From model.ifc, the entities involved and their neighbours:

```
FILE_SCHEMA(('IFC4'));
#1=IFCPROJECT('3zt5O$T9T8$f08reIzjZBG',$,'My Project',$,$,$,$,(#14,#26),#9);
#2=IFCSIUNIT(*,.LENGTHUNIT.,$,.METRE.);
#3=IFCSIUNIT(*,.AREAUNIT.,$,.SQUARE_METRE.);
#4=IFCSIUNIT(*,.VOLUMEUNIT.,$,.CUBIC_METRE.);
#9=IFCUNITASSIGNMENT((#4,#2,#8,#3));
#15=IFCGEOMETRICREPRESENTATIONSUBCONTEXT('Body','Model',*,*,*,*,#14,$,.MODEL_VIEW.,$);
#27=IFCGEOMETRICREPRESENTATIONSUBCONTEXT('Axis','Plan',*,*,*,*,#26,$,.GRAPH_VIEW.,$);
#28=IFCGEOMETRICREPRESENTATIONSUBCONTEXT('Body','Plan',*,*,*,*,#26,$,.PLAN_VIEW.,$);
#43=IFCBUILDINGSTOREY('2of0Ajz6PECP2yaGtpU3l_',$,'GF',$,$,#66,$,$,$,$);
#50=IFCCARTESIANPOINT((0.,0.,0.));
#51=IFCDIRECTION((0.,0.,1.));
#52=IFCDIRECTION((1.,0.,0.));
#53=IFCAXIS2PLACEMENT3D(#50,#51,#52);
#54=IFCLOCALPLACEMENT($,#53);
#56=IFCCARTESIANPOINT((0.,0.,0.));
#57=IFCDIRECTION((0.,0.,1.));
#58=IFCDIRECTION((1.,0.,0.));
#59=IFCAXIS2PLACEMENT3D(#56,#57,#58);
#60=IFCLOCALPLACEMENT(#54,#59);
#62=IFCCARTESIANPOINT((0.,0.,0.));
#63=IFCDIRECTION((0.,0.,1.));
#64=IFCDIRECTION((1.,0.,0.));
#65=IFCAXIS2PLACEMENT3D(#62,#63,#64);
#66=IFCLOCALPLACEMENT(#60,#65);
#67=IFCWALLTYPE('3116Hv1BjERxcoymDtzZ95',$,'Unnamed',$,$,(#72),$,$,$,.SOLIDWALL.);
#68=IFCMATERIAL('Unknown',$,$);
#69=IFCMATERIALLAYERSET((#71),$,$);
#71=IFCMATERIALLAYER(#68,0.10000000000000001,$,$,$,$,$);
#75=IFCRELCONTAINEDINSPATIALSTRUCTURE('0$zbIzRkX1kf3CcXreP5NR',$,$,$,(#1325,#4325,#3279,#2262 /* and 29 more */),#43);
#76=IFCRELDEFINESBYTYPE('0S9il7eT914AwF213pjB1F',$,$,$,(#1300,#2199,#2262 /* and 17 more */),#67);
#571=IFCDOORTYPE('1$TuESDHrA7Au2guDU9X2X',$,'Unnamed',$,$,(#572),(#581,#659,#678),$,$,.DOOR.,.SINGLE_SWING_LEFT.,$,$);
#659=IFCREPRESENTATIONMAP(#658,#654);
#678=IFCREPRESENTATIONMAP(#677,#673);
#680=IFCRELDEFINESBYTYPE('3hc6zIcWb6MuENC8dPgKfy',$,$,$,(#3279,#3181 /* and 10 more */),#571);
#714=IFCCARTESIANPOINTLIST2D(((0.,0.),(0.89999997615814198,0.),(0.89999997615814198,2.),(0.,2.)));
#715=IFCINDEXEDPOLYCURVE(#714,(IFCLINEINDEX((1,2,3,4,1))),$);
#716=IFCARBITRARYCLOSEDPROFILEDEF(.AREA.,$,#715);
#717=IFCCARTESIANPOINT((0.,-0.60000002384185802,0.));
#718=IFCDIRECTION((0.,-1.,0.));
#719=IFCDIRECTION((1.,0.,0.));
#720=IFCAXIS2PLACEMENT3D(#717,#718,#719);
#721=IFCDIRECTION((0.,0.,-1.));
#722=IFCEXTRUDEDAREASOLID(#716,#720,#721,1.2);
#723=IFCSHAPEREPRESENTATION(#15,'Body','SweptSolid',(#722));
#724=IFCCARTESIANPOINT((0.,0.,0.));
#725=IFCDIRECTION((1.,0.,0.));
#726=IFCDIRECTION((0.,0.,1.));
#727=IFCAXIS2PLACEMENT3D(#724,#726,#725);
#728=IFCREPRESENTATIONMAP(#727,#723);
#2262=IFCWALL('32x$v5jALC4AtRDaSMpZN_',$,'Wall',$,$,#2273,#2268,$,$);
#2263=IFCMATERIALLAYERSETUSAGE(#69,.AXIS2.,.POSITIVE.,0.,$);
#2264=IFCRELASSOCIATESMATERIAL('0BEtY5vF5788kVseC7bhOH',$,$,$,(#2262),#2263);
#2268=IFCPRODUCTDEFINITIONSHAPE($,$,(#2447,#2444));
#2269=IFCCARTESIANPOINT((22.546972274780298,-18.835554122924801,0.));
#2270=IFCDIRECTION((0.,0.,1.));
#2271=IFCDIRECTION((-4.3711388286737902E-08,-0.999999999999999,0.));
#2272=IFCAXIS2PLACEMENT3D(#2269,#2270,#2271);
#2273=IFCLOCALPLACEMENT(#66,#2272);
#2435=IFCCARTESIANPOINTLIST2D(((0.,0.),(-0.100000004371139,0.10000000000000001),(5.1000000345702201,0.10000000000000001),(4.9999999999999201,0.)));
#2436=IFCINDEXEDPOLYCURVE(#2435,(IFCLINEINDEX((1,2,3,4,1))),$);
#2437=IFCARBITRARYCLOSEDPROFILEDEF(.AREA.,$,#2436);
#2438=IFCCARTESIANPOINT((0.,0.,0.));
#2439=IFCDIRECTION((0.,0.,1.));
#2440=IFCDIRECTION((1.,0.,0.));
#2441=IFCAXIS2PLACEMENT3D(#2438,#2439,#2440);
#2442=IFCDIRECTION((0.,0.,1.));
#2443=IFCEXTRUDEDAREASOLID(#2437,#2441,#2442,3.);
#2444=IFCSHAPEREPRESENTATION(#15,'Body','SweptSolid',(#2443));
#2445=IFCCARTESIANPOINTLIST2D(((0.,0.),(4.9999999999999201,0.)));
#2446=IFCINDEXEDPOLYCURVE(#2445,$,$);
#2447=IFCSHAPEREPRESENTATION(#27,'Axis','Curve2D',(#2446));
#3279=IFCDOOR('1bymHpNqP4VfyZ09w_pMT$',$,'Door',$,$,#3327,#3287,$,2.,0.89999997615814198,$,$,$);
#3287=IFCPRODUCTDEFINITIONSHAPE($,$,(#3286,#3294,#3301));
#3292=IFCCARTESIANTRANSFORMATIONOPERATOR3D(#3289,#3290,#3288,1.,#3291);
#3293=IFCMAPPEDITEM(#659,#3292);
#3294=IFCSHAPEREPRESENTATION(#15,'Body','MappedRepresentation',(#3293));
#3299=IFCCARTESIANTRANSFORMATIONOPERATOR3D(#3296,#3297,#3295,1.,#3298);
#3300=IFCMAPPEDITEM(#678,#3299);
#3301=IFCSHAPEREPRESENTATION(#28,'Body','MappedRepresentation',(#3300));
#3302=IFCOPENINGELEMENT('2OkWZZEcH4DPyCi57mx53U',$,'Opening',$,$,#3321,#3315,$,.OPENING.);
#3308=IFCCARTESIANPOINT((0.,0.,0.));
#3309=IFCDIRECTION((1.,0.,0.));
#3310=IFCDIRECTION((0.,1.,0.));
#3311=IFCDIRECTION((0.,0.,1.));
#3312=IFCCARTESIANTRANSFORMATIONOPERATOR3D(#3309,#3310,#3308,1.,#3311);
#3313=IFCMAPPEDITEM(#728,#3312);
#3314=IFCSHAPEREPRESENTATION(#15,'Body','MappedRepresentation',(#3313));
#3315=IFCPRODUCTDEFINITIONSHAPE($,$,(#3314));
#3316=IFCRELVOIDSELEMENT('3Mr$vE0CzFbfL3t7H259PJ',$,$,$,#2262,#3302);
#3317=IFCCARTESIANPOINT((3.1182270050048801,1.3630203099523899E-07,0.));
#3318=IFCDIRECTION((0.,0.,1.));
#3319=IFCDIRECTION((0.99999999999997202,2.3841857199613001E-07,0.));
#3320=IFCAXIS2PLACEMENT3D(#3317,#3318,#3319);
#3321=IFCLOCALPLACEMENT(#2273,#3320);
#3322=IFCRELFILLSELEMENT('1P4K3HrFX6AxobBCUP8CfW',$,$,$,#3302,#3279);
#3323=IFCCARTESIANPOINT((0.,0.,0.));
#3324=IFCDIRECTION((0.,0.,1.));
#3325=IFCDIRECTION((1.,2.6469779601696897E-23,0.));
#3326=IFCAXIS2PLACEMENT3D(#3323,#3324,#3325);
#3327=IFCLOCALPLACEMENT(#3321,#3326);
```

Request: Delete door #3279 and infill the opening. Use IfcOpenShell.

```python
import ifcopenshell
import ifcopenshell.api.feature
import ifcopenshell.api.root
import ifcopenshell.geom
import ifcopenshell.util.shape

model = ifcopenshell.open("model.ifc")
settings = ifcopenshell.geom.settings()


def volume(element):
    """Net volume in cubic metres, openings subtracted."""
    shape = ifcopenshell.geom.create_shape(settings, element)
    return ifcopenshell.util.shape.get_volume(shape.geometry)


door = model.by_guid("1bymHpNqP4VfyZ09w_pMT$")
opening = door.FillsVoids[0].RelatingOpeningElement
wall = opening.VoidsElements[0].RelatingBuildingElement
before = volume(wall)

ifcopenshell.api.root.remove_product(model, product=door)
ifcopenshell.api.feature.remove_feature(model, feature=opening)

after = volume(wall)

print(f"wall volume {before:.3f} -> {after:.3f} m3")

model.write("model_edited.ifc")
```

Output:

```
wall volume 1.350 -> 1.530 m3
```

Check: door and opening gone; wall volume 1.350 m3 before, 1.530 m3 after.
